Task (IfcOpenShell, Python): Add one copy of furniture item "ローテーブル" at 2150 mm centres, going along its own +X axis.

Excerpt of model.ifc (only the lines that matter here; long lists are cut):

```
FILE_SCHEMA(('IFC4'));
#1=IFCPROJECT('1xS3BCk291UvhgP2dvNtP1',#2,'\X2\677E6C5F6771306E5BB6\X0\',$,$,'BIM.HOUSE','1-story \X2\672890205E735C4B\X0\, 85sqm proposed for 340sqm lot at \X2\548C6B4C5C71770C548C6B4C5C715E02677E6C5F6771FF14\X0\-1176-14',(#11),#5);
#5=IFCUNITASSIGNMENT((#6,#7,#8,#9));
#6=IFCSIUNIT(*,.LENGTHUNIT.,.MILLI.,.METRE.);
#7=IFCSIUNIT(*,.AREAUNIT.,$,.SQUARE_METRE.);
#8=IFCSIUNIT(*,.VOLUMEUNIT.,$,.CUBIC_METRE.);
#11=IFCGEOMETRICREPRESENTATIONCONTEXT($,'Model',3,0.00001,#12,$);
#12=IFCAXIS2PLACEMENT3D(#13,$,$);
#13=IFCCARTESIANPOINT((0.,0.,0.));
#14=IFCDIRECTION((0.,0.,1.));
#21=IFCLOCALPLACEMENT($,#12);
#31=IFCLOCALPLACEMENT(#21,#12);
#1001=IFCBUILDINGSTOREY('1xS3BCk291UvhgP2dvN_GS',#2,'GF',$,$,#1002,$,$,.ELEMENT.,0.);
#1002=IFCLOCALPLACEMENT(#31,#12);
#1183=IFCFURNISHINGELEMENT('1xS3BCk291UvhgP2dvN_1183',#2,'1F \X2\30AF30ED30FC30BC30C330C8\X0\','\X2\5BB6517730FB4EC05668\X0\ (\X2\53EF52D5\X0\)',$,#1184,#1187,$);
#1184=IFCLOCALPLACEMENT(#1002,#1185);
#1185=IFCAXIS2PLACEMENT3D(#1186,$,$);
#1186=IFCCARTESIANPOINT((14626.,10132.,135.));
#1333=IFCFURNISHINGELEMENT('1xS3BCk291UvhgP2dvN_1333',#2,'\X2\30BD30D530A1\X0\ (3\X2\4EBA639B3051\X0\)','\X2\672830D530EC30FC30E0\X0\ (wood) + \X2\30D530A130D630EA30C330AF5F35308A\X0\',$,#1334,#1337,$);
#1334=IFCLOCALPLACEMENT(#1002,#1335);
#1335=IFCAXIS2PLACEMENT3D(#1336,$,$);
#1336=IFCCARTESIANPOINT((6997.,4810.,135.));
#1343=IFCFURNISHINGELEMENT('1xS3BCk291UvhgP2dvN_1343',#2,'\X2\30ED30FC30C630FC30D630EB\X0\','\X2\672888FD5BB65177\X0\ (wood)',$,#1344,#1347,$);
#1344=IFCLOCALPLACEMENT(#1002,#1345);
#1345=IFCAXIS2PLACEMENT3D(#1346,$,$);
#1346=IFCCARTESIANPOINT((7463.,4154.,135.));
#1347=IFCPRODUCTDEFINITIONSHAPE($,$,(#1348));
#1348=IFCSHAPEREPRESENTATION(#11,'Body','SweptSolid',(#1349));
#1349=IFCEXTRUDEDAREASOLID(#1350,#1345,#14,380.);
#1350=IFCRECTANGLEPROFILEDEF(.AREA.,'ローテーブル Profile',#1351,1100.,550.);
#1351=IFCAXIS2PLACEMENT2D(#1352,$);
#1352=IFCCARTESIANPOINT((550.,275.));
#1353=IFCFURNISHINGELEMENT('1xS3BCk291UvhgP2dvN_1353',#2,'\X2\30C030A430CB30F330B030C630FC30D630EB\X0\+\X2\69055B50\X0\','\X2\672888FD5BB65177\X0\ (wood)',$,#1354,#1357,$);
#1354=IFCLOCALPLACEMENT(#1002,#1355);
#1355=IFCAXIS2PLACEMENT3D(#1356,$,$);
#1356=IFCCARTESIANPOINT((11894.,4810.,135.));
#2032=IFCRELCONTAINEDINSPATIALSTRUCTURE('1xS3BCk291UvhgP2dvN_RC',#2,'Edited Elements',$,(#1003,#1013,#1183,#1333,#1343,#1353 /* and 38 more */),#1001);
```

```python
import ifcopenshell
import ifcopenshell.api.geometry
import ifcopenshell.api.root
import ifcopenshell.util.element
import ifcopenshell.util.placement

model = ifcopenshell.open("model.ifc")


def reuse_history(source, copy):
    """copy_class also copies each property set's owner history, people and application; keep the originals."""
    for rel in copy.IsDefinedBy:
        if rel.is_a("IfcRelDefinesByProperties") and (history := rel.RelatingPropertyDefinition.OwnerHistory):
            rel.RelatingPropertyDefinition.OwnerHistory = source.OwnerHistory
            ifcopenshell.util.element.remove_deep2(model, history)


source = model.by_id(1343)
base = ifcopenshell.util.placement.get_local_placement(source.ObjectPlacement)
step = base[:3, 0] * 2150.0

for i in range(1, 2):
    copy = ifcopenshell.api.root.copy_class(model, product=source)
    copy.Representation = ifcopenshell.util.element.copy_deep(
        model, source.Representation, exclude=["IfcGeometricRepresentationContext", "IfcRepresentationMap"]
    )
    reuse_history(source, copy)
    matrix = base.copy()
    matrix[:3, 3] += i * step
    print("added at", matrix[:3, 3].round(3) + 0.0)
    ifcopenshell.api.geometry.edit_object_placement(model, product=copy, matrix=matrix, is_si=False)

model.write("model_v2.ifc")
```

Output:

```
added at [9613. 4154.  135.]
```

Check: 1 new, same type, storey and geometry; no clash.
